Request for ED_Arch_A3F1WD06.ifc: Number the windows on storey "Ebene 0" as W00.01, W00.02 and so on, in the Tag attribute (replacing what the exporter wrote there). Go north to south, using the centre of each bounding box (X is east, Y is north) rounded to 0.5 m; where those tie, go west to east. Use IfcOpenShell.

First a look at what the model holds.

```python
import ifcopenshell
import ifcopenshell.util.element
import ifcopenshell.util.placement

model = ifcopenshell.open("ED_Arch_A3F1WD06.ifc")
print(model.schema)
storey = next(s for s in model.by_type("IfcBuildingStorey") if s.Name == "Ebene 0")
windows = [e for e in ifcopenshell.util.element.get_decomposition(storey) if e.is_a("IfcWindow")]
for e in sorted(windows, key=lambda e: e.id()):
    origin = ifcopenshell.util.placement.get_local_placement(e.ObjectPlacement)[:3, 3]
    print(e.id(), e.Tag, e.Name, origin.round(2) + 0.0, sep=" | ")
```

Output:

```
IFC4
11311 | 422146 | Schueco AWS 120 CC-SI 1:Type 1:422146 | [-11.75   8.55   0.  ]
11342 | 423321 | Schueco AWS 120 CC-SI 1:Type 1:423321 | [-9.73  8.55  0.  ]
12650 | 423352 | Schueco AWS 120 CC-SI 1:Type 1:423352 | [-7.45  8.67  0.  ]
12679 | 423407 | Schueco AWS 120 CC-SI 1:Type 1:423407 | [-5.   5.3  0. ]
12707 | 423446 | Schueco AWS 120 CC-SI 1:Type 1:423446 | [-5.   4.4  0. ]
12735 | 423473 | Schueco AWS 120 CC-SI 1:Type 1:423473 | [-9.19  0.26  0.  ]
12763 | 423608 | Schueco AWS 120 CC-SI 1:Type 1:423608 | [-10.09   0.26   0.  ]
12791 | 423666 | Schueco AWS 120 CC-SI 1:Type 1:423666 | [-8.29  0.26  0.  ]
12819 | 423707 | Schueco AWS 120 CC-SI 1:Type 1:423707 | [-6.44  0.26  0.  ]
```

```python
import ifcopenshell
import ifcopenshell.geom
import ifcopenshell.util.element
import ifcopenshell.util.shape

model = ifcopenshell.open("ED_Arch_A3F1WD06.ifc")
settings = ifcopenshell.geom.settings()
settings.set("use-world-coords", True)


def centre(element):
    shape = ifcopenshell.geom.create_shape(settings, element)
    return ifcopenshell.util.shape.get_bbox_centroid(shape.geometry)


storey = next(s for s in model.by_type("IfcBuildingStorey") if s.Name == "Ebene 0")
windows = [e for e in ifcopenshell.util.element.get_decomposition(storey) if e.is_a("IfcWindow")]

# Insertion points can sit at a corner or the storey origin, so sort by the geometry (in metres).
centres = {e: centre(e) for e in windows}
windows.sort(key=lambda e: (-round(centres[e][1] / 0.5), centres[e][0]))

for i, e in enumerate(windows, start=1):
    number = f"W00.{i:02d}"
    e.Tag = number
    print(e.id(), number)

model.write("ED_Arch_A3F1WD06_rev.ifc")
```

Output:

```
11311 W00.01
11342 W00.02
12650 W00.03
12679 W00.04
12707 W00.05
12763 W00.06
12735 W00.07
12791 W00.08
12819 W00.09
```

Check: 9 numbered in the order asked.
